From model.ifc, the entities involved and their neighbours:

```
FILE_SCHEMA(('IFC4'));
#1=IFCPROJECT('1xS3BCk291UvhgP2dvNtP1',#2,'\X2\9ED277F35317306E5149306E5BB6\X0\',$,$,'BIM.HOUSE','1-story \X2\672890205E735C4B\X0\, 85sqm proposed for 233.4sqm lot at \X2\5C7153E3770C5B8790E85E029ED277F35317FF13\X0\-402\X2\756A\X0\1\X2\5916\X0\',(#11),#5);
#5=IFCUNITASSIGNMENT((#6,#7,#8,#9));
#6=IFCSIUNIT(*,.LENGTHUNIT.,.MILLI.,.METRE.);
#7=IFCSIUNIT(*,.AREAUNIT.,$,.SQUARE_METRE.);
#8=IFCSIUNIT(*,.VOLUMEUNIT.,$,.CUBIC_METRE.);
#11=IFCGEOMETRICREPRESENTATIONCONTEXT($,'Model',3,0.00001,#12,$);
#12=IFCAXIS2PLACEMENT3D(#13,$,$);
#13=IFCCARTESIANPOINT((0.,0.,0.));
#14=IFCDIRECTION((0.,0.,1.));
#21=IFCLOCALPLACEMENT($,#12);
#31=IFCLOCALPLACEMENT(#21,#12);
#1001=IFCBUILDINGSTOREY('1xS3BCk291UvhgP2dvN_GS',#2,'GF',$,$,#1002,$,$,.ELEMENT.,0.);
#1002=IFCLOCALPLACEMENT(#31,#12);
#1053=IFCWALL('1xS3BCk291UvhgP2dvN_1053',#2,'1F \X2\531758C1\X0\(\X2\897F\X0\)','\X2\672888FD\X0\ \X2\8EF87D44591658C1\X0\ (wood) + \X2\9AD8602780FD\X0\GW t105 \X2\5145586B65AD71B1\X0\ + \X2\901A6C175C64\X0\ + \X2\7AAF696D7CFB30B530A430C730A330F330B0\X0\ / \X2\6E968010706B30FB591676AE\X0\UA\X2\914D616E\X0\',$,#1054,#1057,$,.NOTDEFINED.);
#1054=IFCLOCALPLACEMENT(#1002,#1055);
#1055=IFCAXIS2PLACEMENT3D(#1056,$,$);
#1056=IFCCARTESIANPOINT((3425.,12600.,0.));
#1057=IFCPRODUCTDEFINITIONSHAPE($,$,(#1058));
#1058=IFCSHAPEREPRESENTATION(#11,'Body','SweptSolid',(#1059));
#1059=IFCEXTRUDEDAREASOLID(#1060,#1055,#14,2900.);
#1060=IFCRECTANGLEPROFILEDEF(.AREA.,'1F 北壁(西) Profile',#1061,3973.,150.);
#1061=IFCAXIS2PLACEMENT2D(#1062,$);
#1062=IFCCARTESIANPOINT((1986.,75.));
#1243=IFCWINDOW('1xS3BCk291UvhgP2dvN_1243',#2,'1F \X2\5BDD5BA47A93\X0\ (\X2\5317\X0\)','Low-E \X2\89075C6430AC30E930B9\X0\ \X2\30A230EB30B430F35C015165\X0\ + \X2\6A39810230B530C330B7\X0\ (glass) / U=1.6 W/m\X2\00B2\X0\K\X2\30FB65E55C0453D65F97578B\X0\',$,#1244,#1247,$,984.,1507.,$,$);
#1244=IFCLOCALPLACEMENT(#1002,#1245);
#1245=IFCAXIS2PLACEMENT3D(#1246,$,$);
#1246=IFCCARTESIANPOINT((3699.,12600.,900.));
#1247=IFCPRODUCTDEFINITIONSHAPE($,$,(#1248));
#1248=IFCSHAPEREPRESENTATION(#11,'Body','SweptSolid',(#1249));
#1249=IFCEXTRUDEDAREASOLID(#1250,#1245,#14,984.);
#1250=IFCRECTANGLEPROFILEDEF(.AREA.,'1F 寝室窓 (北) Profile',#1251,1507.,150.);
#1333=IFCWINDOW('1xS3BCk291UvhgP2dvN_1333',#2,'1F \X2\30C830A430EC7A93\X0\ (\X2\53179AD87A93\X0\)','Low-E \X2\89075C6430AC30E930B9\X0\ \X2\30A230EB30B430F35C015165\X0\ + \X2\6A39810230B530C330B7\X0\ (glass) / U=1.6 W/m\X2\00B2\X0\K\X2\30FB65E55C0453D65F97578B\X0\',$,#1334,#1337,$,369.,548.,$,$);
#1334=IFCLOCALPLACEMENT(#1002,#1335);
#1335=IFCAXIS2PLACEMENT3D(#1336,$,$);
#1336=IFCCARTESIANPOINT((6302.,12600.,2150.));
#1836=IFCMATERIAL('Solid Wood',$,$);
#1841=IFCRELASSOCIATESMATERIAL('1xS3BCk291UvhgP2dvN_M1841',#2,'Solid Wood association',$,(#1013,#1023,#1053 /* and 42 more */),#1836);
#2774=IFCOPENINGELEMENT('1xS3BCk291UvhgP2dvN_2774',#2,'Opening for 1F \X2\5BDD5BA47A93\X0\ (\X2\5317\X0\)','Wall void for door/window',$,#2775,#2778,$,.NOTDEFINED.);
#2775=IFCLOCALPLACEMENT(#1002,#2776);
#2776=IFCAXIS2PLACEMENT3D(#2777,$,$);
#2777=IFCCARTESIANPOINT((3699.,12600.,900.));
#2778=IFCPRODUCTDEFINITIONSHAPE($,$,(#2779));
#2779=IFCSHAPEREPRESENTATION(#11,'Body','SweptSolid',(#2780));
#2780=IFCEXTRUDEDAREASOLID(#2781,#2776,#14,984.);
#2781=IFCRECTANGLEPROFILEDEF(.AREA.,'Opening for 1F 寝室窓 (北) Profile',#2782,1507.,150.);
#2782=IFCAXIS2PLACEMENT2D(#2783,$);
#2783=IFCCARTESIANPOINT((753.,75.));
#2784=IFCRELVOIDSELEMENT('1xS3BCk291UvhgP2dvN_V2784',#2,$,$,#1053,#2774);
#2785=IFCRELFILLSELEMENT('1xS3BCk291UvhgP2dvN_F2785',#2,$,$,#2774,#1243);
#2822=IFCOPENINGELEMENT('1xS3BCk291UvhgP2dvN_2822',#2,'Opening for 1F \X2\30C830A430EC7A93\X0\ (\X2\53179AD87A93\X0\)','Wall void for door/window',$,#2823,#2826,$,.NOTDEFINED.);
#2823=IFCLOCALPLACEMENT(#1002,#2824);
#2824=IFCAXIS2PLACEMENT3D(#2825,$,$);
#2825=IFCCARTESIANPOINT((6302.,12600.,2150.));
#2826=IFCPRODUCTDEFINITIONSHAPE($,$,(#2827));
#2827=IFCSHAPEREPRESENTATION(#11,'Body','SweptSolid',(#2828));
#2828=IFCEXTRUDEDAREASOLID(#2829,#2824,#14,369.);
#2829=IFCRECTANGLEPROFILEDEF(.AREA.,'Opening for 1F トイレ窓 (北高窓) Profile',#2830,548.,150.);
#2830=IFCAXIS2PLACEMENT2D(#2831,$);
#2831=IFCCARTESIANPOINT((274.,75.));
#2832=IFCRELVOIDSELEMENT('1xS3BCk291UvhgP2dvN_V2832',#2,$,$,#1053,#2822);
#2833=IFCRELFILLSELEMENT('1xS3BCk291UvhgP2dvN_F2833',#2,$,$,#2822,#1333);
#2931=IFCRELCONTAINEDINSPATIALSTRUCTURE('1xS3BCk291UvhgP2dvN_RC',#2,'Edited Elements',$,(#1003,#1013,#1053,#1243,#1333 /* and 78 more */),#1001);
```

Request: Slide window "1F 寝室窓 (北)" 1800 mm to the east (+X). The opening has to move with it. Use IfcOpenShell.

```python
import ifcopenshell
import ifcopenshell.api.geometry
import ifcopenshell.util.placement
import ifcopenshell.util.unit

model = ifcopenshell.open("model.ifc")
unit_scale = ifcopenshell.util.unit.calculate_unit_scale(model)

window = model.by_guid("1xS3BCk291UvhgP2dvN_1243")
opening = window.FillsVoids[0].RelatingOpeningElement
wall = opening.VoidsElements[0].RelatingBuildingElement

wall_matrix = ifcopenshell.util.placement.get_local_placement(wall.ObjectPlacement)
shift = wall_matrix[:3, 0] * 1.8 / unit_scale
before = ifcopenshell.util.placement.get_local_placement(window.ObjectPlacement)[:3, 3].copy()

# The window is not placed relative to its opening, so move both.
for product in (opening, window):
    matrix = ifcopenshell.util.placement.get_local_placement(product.ObjectPlacement)
    matrix[:3, 3] += shift
    ifcopenshell.api.geometry.edit_object_placement(model, product=product, matrix=matrix, is_si=False)

after = ifcopenshell.util.placement.get_local_placement(window.ObjectPlacement)[:3, 3]
print("window moved by", (after - before).round(3) + 0.0)

model.write("model_edited.ifc")
```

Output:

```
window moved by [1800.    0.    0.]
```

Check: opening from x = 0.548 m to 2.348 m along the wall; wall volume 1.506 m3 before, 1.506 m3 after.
